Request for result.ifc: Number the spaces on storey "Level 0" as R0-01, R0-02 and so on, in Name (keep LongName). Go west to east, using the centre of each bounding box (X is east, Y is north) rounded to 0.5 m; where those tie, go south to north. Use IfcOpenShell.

First a look at what the model holds.

```python
import ifcopenshell
import ifcopenshell.util.element
import ifcopenshell.util.placement

model = ifcopenshell.open("result.ifc")
print(model.schema)
storey = next(s for s in model.by_type("IfcBuildingStorey") if s.Name == "Level 0")
spaces = [e for e in ifcopenshell.util.element.get_decomposition(storey) if e.is_a("IfcSpace")]
for e in sorted(spaces, key=lambda e: e.id()):
    origin = ifcopenshell.util.placement.get_local_placement(e.ObjectPlacement)[:3, 3]
    print(e.id(), e.Name, e.LongName, origin.round(2) + 0.0, sep=" | ")
```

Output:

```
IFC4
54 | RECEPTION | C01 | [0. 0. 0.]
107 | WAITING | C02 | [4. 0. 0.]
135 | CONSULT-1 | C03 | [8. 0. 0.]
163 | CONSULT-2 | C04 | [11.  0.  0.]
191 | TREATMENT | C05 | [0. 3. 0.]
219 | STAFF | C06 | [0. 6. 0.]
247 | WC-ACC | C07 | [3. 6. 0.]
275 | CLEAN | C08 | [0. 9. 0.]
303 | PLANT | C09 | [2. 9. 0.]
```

```python
import ifcopenshell
import ifcopenshell.geom
import ifcopenshell.util.element
import ifcopenshell.util.shape

model = ifcopenshell.open("result.ifc")
settings = ifcopenshell.geom.settings()
settings.set("use-world-coords", True)


def centre(element):
    shape = ifcopenshell.geom.create_shape(settings, element)
    return ifcopenshell.util.shape.get_bbox_centroid(shape.geometry)


storey = next(s for s in model.by_type("IfcBuildingStorey") if s.Name == "Level 0")
spaces = [e for e in ifcopenshell.util.element.get_decomposition(storey) if e.is_a("IfcSpace")]

# Insertion points can sit at a corner or the storey origin, so sort by the geometry (in metres).
centres = {e: centre(e) for e in spaces}
spaces.sort(key=lambda e: (round(centres[e][0] / 0.5), centres[e][1]))

for i, e in enumerate(spaces, start=1):
    number = f"R0-{i:02d}"
    e.Name = number
    print(e.id(), number)

model.write("result_rev.ifc")
```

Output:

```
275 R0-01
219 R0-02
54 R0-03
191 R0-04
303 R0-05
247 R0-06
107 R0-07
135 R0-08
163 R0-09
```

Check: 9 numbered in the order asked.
